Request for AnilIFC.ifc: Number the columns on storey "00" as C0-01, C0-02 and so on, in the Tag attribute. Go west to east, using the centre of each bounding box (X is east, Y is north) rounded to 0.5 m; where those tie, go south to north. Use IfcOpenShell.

First a look at what the model holds.

```python
import ifcopenshell
import ifcopenshell.util.element
import ifcopenshell.util.placement

model = ifcopenshell.open("AnilIFC.ifc")
print(model.schema)
storey = next(s for s in model.by_type("IfcBuildingStorey") if s.Name == "00")
columns = [e for e in ifcopenshell.util.element.get_decomposition(storey) if e.is_a("IfcColumn")]
for e in sorted(columns, key=lambda e: e.id()):
    origin = ifcopenshell.util.placement.get_local_placement(e.ObjectPlacement)[:3, 3]
    print(e.id(), e.Tag, e.Name, origin.round(2) + 0.0, sep=" | ")
```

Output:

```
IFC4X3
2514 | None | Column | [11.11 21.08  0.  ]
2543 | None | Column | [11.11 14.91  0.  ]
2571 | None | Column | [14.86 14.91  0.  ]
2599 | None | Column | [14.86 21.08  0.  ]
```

```python
import ifcopenshell
import ifcopenshell.geom
import ifcopenshell.util.element
import ifcopenshell.util.shape

model = ifcopenshell.open("AnilIFC.ifc")
settings = ifcopenshell.geom.settings()
settings.set("use-world-coords", True)


def centre(element):
    shape = ifcopenshell.geom.create_shape(settings, element)
    return ifcopenshell.util.shape.get_bbox_centroid(shape.geometry)


storey = next(s for s in model.by_type("IfcBuildingStorey") if s.Name == "00")
columns = [e for e in ifcopenshell.util.element.get_decomposition(storey) if e.is_a("IfcColumn")]

# Insertion points can sit at a corner or the storey origin, so sort by the geometry (in metres).
centres = {e: centre(e) for e in columns}
columns.sort(key=lambda e: (round(centres[e][0] / 0.5), centres[e][1]))

for i, e in enumerate(columns, start=1):
    number = f"C0-{i:02d}"
    e.Tag = number
    print(e.id(), number)

model.write("AnilIFC_edited.ifc")
```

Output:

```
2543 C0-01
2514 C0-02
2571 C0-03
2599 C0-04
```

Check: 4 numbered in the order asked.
